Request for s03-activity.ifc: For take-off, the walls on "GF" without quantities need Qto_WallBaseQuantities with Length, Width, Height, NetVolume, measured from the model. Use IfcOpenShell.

First a look at what the model holds.

```python
import ifcopenshell
import ifcopenshell.util.element
import ifcopenshell.util.unit

model = ifcopenshell.open("s03-activity.ifc")
print(model.schema)
for unit_type in ("LENGTHUNIT", "AREAUNIT", "VOLUMEUNIT"):
    print(unit_type, ifcopenshell.util.unit.calculate_unit_scale(model, unit_type))
storey = next(s for s in model.by_type("IfcBuildingStorey") if s.Name == "GF")
walls = [e for e in ifcopenshell.util.element.get_decomposition(storey) if e.is_a("IfcWall")]
for e in sorted(walls, key=lambda e: e.id()):
    print(e.id(), e.is_a(), e.Name, list(ifcopenshell.util.element.get_psets(e, qtos_only=True)), sep=" | ")
```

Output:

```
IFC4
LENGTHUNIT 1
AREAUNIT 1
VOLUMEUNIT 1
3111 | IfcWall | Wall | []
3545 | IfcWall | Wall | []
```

```python
import ifcopenshell
import ifcopenshell.api.pset
import ifcopenshell.geom
import ifcopenshell.util.element
import ifcopenshell.util.shape
import ifcopenshell.util.unit

model = ifcopenshell.open("s03-activity.ifc")
unit_scale = ifcopenshell.util.unit.calculate_unit_scale(model)
volume_scale = ifcopenshell.util.unit.calculate_unit_scale(model, "VOLUMEUNIT")
settings = ifcopenshell.geom.settings()

storey = next(s for s in model.by_type("IfcBuildingStorey") if s.Name == "GF")
walls = [e for e in ifcopenshell.util.element.get_decomposition(storey) if e.is_a("IfcWall")]

for e in sorted(walls, key=lambda e: e.id()):
    if ifcopenshell.util.element.get_psets(e, qtos_only=True, should_inherit=False):
        continue
    # Geometry comes back in metres, in the element's own axes.
    shape = ifcopenshell.geom.create_shape(settings, e)
    values = {
        "Length": ifcopenshell.util.shape.get_x(shape.geometry) / unit_scale,
        "Width": ifcopenshell.util.shape.get_y(shape.geometry) / unit_scale,
        "Height": ifcopenshell.util.shape.get_z(shape.geometry) / unit_scale,
        "NetVolume": ifcopenshell.util.shape.get_volume(shape.geometry) / volume_scale,
    }
    qto = ifcopenshell.api.pset.add_qto(model, product=e, name="Qto_WallBaseQuantities")
    ifcopenshell.api.pset.edit_qto(model, qto=qto, properties=values)
    print(e.id(), {k: round(v, 3) for k, v in values.items()})

model.write("s03-activity_v2.ifc")
```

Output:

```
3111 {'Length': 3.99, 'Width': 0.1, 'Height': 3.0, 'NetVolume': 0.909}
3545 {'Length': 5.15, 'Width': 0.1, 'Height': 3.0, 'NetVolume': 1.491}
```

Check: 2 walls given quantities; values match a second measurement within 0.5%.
